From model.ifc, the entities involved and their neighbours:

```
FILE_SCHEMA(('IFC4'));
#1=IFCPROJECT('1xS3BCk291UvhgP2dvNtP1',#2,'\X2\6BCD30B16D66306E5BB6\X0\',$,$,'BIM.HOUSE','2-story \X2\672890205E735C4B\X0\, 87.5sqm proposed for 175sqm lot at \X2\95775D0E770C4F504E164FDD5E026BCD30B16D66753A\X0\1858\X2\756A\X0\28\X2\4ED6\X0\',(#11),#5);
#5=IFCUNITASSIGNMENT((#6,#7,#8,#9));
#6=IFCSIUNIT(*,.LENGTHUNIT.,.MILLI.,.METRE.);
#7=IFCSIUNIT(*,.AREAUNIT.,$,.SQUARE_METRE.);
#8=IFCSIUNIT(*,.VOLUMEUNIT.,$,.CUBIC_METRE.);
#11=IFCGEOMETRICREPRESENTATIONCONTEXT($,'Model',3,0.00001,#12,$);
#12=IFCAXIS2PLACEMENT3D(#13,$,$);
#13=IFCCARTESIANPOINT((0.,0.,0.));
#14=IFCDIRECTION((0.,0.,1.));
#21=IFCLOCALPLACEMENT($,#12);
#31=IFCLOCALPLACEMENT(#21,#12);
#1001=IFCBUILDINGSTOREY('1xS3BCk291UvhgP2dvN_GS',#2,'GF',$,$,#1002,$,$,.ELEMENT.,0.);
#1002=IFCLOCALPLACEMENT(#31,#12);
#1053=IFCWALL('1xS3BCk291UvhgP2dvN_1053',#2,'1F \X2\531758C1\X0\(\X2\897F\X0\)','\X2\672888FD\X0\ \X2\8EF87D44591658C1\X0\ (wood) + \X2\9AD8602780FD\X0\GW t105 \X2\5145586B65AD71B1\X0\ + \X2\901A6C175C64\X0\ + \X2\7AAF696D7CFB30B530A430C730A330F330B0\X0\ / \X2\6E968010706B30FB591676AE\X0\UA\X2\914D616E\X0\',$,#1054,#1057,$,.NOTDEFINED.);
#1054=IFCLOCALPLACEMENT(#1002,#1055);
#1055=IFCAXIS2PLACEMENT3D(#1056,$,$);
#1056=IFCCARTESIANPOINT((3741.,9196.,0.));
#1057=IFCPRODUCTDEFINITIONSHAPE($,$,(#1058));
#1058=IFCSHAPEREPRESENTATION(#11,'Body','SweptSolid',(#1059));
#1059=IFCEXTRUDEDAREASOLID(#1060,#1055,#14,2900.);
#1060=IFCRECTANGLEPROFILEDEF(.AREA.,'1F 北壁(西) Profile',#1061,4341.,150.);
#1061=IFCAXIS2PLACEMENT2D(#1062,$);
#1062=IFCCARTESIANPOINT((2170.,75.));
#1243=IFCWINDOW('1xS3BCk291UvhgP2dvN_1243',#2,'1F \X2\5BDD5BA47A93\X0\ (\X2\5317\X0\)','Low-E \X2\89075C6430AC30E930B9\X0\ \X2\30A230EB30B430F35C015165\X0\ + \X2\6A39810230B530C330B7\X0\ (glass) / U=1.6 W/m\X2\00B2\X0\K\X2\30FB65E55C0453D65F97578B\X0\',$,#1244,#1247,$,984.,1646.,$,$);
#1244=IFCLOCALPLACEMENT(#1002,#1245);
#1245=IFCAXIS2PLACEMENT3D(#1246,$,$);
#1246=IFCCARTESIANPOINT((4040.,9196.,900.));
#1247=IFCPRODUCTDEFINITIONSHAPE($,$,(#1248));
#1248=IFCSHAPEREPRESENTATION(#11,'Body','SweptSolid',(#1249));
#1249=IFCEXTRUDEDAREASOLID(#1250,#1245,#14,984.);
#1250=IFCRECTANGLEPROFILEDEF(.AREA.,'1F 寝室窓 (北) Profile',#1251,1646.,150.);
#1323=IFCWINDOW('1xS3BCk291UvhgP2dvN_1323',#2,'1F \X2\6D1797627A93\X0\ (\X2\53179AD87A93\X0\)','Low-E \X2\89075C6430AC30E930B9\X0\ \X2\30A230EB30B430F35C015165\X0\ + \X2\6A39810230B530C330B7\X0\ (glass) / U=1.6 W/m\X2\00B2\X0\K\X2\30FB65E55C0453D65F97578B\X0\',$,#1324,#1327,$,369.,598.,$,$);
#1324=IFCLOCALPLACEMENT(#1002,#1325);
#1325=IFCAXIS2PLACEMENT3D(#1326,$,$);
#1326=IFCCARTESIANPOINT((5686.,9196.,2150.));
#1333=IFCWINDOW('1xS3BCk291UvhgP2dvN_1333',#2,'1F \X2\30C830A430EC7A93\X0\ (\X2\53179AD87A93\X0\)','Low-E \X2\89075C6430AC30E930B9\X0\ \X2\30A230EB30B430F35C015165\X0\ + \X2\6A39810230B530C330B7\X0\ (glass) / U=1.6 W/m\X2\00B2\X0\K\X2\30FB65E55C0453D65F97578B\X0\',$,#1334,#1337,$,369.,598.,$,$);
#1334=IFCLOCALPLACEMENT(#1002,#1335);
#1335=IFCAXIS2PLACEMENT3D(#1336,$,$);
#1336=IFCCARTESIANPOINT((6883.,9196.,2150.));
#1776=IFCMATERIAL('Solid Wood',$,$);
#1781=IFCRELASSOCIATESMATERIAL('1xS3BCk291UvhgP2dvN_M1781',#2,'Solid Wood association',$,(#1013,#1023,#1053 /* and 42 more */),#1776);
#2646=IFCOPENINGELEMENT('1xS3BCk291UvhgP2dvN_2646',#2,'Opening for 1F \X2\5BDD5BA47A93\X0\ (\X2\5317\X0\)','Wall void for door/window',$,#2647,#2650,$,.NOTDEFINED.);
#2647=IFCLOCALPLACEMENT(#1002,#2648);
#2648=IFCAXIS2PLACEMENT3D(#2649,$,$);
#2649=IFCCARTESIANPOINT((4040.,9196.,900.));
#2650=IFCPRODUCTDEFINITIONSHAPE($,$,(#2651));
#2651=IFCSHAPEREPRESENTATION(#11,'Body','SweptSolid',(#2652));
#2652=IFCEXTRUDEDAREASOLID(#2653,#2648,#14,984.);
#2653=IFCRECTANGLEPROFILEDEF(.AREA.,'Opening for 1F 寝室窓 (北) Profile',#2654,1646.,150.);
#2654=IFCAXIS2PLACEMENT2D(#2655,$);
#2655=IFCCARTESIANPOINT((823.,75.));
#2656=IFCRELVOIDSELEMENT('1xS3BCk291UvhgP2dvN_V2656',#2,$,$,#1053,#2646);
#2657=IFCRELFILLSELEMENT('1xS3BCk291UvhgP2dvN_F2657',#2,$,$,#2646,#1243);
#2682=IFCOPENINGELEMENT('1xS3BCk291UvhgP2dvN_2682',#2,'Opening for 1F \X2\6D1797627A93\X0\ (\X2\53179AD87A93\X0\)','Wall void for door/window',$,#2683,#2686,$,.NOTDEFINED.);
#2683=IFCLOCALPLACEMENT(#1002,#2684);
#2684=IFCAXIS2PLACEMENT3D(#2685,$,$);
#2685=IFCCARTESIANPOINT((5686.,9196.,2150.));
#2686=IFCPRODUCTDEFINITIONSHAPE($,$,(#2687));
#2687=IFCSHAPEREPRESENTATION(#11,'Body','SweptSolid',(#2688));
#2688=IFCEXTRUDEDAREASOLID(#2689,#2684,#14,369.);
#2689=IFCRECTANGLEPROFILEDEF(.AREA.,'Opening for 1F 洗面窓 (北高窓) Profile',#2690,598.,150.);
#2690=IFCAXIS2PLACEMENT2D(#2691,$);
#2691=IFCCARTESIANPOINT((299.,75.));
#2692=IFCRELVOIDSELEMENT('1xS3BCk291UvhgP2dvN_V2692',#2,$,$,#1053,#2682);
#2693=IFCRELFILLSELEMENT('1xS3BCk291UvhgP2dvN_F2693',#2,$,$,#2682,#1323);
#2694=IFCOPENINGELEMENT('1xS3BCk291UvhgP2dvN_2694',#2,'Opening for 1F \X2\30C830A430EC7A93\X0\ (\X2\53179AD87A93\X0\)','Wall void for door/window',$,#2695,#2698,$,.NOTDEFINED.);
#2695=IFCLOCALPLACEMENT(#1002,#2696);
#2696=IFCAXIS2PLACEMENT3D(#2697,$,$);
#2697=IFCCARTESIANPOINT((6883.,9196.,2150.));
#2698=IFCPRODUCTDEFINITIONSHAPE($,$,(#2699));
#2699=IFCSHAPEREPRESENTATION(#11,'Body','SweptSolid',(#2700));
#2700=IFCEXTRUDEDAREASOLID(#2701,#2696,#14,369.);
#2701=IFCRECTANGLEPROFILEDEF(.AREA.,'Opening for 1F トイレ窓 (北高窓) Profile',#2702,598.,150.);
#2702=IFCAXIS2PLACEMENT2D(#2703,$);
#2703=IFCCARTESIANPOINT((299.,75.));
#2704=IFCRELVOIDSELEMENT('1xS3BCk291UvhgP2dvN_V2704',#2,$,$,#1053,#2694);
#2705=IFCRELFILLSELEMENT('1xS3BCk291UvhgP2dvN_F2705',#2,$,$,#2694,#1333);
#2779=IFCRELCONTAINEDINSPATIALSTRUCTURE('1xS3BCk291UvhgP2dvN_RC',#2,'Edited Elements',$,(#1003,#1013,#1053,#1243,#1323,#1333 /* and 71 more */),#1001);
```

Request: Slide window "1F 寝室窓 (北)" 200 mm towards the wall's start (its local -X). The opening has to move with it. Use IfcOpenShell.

```python
import ifcopenshell
import ifcopenshell.api.geometry
import ifcopenshell.util.placement
import ifcopenshell.util.unit

model = ifcopenshell.open("model.ifc")
unit_scale = ifcopenshell.util.unit.calculate_unit_scale(model)

window = model.by_guid("1xS3BCk291UvhgP2dvN_1243")
opening = window.FillsVoids[0].RelatingOpeningElement
wall = opening.VoidsElements[0].RelatingBuildingElement

wall_matrix = ifcopenshell.util.placement.get_local_placement(wall.ObjectPlacement)
shift = wall_matrix[:3, 0] * -0.2 / unit_scale
before = ifcopenshell.util.placement.get_local_placement(window.ObjectPlacement)[:3, 3].copy()

# The window is not placed relative to its opening, so move both.
for product in (opening, window):
    matrix = ifcopenshell.util.placement.get_local_placement(product.ObjectPlacement)
    matrix[:3, 3] += shift
    ifcopenshell.api.geometry.edit_object_placement(model, product=product, matrix=matrix, is_si=False)

after = ifcopenshell.util.placement.get_local_placement(window.ObjectPlacement)[:3, 3]
print("window moved by", (after - before).round(3) + 0.0)

model.write("model_edited.ifc")
```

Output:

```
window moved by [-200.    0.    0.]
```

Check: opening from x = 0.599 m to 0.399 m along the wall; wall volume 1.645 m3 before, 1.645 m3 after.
